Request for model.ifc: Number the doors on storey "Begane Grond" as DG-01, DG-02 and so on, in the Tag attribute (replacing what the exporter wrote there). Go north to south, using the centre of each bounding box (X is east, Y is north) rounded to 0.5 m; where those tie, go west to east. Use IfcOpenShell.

First a look at what the model holds.

```python
import ifcopenshell
import ifcopenshell.util.element
import ifcopenshell.util.placement

model = ifcopenshell.open("model.ifc")
print(model.schema)
storey = next(s for s in model.by_type("IfcBuildingStorey") if s.Name == "Begane Grond")
doors = [e for e in ifcopenshell.util.element.get_decomposition(storey) if e.is_a("IfcDoor")]
for e in sorted(doors, key=lambda e: e.id()):
    origin = ifcopenshell.util.placement.get_local_placement(e.ObjectPlacement)[:3, 3]
    print(e.id(), e.Tag, e.Name, origin.round(2) + 0.0, sep=" | ")
```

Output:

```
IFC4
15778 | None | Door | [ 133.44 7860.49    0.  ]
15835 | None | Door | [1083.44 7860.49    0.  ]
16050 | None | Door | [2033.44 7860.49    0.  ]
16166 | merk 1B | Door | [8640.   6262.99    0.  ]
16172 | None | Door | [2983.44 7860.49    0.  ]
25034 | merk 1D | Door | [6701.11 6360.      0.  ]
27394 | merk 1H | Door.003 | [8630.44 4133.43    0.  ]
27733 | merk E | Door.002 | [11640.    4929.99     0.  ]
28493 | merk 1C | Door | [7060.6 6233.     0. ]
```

```python
import ifcopenshell
import ifcopenshell.geom
import ifcopenshell.util.element
import ifcopenshell.util.shape

model = ifcopenshell.open("model.ifc")
settings = ifcopenshell.geom.settings()
settings.set("use-world-coords", True)


def centre(element):
    shape = ifcopenshell.geom.create_shape(settings, element)
    return ifcopenshell.util.shape.get_bbox_centroid(shape.geometry)


storey = next(s for s in model.by_type("IfcBuildingStorey") if s.Name == "Begane Grond")
doors = [e for e in ifcopenshell.util.element.get_decomposition(storey) if e.is_a("IfcDoor")]

# Insertion points can sit at a corner or the storey origin, so sort by the geometry (in metres).
centres = {e: centre(e) for e in doors}
doors.sort(key=lambda e: (-round(centres[e][1] / 0.5), centres[e][0]))

for i, e in enumerate(doors, start=1):
    number = f"DG-{i:02d}"
    e.Tag = number
    print(e.id(), number)

model.write("model_v2.ifc")
```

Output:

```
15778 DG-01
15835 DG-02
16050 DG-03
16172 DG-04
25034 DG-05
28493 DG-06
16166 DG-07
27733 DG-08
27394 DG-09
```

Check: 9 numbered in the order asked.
